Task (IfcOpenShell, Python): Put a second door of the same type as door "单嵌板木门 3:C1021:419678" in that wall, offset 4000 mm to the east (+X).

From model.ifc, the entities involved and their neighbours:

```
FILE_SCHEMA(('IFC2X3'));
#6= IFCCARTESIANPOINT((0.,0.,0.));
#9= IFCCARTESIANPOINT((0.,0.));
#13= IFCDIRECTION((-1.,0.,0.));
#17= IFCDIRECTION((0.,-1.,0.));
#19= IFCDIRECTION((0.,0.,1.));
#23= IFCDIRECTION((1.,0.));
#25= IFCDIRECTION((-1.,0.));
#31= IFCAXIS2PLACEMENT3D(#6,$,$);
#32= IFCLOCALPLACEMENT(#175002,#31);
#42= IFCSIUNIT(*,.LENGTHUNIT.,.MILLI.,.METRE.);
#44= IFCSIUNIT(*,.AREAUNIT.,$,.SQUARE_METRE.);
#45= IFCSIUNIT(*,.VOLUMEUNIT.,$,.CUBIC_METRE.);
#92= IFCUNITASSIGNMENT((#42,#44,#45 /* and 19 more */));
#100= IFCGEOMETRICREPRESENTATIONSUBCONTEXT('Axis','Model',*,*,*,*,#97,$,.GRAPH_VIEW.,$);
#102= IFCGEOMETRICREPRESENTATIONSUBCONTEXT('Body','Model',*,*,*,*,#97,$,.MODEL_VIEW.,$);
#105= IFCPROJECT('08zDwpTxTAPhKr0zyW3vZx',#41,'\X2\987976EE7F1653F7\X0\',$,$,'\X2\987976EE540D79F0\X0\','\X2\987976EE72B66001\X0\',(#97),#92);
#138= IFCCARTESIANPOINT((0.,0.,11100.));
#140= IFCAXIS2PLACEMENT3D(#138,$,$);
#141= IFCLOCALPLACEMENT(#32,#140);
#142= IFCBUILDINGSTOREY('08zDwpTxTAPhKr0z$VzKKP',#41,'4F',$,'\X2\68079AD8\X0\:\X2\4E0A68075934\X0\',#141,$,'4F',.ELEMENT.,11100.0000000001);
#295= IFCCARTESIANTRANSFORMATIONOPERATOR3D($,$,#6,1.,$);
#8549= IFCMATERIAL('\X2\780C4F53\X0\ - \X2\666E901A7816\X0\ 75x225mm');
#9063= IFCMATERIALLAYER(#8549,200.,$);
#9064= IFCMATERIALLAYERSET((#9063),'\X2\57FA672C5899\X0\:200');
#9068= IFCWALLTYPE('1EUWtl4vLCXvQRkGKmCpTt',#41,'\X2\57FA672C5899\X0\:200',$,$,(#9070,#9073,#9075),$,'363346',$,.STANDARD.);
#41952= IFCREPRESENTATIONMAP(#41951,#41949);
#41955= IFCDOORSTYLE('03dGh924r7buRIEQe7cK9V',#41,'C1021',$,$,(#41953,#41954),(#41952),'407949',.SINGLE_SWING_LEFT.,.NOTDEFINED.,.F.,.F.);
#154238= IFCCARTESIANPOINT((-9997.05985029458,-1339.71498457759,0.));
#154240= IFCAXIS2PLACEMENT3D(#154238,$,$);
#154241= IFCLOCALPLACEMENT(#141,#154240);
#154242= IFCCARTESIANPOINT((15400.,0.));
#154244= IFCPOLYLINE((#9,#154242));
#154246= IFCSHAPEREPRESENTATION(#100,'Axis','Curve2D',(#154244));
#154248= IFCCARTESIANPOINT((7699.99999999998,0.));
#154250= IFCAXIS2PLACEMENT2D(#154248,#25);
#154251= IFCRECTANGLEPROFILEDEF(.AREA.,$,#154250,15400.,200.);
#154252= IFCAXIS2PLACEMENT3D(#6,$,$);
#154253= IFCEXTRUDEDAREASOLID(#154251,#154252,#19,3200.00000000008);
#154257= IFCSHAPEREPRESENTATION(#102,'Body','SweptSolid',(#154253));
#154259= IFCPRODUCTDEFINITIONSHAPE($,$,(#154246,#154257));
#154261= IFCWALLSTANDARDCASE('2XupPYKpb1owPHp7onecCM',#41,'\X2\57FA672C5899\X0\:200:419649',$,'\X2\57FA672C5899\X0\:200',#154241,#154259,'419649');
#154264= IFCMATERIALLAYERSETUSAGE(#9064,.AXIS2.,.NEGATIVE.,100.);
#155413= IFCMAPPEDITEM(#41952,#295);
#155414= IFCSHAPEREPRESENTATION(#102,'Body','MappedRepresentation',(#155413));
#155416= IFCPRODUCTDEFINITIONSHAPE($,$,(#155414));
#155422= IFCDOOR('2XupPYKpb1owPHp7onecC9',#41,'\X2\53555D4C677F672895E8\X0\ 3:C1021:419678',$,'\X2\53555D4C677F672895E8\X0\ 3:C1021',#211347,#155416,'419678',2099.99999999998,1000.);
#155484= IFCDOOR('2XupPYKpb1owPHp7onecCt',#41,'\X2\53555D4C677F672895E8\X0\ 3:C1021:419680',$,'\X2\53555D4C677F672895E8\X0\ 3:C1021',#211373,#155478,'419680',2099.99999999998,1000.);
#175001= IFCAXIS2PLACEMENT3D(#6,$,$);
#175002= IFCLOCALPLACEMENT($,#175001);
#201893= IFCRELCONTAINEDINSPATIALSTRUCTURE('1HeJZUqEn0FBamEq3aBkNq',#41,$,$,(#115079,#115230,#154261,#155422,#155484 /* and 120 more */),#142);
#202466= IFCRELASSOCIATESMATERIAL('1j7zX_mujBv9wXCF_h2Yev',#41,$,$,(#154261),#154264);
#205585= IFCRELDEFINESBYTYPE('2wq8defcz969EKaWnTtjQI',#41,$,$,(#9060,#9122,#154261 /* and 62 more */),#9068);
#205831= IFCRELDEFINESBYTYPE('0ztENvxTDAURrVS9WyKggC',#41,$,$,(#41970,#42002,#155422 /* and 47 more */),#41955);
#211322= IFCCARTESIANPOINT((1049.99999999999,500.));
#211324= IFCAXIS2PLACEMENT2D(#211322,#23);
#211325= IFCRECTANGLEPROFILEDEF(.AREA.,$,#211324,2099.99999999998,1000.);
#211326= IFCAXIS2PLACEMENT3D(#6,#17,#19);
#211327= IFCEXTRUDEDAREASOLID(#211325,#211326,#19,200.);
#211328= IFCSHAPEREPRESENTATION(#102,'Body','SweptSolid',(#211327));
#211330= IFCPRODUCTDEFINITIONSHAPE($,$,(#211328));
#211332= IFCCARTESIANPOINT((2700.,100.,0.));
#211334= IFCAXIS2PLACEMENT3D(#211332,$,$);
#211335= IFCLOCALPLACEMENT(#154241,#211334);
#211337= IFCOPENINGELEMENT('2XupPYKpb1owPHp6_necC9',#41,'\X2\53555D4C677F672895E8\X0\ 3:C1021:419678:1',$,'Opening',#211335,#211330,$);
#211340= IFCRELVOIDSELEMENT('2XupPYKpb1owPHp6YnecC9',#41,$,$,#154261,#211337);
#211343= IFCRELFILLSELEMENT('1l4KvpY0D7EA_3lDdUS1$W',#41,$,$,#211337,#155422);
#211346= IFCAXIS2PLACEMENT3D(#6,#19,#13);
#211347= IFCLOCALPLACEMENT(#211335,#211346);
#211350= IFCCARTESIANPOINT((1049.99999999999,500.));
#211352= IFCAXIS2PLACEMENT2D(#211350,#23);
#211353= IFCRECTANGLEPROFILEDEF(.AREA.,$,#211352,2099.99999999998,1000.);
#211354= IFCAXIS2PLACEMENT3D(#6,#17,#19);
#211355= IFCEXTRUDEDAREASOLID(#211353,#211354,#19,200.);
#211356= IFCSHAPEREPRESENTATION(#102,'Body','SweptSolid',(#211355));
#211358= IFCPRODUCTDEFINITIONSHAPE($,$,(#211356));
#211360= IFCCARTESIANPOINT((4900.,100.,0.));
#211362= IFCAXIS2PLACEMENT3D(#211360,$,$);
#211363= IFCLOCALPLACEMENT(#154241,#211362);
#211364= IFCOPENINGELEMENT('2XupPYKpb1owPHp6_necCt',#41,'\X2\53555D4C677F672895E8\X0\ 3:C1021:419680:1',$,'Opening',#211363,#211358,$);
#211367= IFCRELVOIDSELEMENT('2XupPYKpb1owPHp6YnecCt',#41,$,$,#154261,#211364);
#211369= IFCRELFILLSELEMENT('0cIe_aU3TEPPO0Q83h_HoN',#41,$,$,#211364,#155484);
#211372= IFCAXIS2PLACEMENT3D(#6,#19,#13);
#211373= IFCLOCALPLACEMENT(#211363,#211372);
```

```python
import ifcopenshell
import ifcopenshell.api.feature
import ifcopenshell.api.geometry
import ifcopenshell.api.root
import ifcopenshell.geom
import ifcopenshell.util.element
import ifcopenshell.util.placement
import ifcopenshell.util.shape
import ifcopenshell.util.unit

model = ifcopenshell.open("model.ifc")
unit_scale = ifcopenshell.util.unit.calculate_unit_scale(model)
settings = ifcopenshell.geom.settings()


def volume(element):
    """Net volume in cubic metres, openings subtracted."""
    shape = ifcopenshell.geom.create_shape(settings, element)
    return ifcopenshell.util.shape.get_volume(shape.geometry)


def reuse_history(source, copy):
    """copy_class also copies each property set's owner history, people and application; keep the originals."""
    for rel in copy.IsDefinedBy:
        if rel.is_a("IfcRelDefinesByProperties") and (history := rel.RelatingPropertyDefinition.OwnerHistory):
            rel.RelatingPropertyDefinition.OwnerHistory = source.OwnerHistory
            ifcopenshell.util.element.remove_deep2(model, history)


door = model.by_id(155422)
opening = door.FillsVoids[0].RelatingOpeningElement
wall = opening.VoidsElements[0].RelatingBuildingElement
before = volume(wall)
shift = ifcopenshell.util.placement.get_local_placement(wall.ObjectPlacement)[:3, 0] * 4 / unit_scale

# copy_class copies the void relationship, type, container and properties, but no geometry.
new_opening = ifcopenshell.api.root.copy_class(model, product=opening)
new_opening.Representation = ifcopenshell.util.element.copy_deep(
    model, opening.Representation, exclude=["IfcGeometricRepresentationContext", "IfcRepresentationMap"]
)
new_opening.Name = "单嵌板木门 3:C1021"
new_door = ifcopenshell.api.root.copy_class(model, product=door)
new_door.Representation = ifcopenshell.util.element.copy_deep(
    model, door.Representation, exclude=["IfcGeometricRepresentationContext", "IfcRepresentationMap"]
)
new_door.Name = "单嵌板木门 3:C1021"
new_door.Tag = None
reuse_history(door, new_door)
fills = ifcopenshell.api.feature.add_filling(model, opening=new_opening, element=new_door)
fills.OwnerHistory = new_door.OwnerHistory  # required in IFC2X3

for old, new in ((opening, new_opening), (door, new_door)):
    matrix = ifcopenshell.util.placement.get_local_placement(old.ObjectPlacement)
    matrix[:3, 3] += shift
    ifcopenshell.api.geometry.edit_object_placement(model, product=new, matrix=matrix, is_si=False)

after = volume(wall)

print(f"wall volume {before:.3f} -> {after:.3f} m3")

model.write("model-out.ifc")
```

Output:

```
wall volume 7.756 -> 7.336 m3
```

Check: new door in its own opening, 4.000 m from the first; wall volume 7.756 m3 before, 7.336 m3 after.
